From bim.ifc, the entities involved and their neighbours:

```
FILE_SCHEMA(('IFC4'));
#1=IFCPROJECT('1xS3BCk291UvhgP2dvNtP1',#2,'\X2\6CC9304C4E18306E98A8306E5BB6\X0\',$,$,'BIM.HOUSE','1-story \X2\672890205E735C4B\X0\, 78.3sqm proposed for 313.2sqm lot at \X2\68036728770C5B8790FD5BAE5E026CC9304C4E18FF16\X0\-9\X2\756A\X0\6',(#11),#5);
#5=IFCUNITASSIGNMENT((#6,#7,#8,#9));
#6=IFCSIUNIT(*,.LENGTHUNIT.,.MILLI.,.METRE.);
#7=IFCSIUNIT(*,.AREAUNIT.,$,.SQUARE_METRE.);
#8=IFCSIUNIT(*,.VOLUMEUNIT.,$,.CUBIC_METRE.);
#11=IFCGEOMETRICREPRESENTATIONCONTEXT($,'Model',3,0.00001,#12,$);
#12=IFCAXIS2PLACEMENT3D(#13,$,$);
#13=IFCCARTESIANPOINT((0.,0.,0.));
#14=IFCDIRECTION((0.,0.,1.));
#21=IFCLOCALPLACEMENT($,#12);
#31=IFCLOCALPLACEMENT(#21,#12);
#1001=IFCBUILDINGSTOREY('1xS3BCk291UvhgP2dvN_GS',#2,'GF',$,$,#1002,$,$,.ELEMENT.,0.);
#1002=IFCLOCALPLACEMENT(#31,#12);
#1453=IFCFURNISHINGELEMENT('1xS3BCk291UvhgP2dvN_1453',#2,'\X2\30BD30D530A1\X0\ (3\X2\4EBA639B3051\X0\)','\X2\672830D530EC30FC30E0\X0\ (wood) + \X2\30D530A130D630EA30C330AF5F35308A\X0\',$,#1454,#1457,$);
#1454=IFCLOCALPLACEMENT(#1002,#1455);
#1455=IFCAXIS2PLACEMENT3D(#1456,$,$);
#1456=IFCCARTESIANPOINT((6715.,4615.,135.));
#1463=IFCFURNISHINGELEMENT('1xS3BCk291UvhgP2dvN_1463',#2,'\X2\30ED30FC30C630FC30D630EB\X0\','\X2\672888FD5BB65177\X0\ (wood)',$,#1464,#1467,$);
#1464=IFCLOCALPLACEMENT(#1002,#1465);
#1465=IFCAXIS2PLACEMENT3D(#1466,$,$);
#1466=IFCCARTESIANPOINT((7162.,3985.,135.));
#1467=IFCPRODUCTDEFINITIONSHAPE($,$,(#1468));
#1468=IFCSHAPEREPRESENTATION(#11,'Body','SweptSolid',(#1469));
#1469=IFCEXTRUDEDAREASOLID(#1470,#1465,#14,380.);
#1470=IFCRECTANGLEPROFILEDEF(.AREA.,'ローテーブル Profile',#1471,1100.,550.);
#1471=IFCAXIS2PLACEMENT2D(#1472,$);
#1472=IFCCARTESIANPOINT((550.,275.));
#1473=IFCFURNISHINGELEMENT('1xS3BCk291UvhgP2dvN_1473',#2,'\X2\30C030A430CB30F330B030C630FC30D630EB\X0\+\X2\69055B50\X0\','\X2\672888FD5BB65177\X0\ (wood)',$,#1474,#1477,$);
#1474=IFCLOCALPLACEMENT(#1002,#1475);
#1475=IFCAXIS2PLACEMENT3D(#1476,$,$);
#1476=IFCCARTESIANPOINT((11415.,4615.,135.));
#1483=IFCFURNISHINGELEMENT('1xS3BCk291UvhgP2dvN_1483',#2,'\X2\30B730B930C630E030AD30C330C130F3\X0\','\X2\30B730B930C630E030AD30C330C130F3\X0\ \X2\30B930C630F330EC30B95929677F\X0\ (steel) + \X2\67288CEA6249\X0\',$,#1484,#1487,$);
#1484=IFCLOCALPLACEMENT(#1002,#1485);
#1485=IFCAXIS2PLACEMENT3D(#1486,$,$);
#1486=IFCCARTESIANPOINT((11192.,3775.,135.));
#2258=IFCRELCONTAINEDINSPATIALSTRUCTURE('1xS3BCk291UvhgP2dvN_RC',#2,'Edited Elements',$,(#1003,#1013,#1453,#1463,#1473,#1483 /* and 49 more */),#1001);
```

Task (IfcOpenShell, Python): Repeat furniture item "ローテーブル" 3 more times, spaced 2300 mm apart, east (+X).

```python
import numpy as np
import ifcopenshell
import ifcopenshell.api.geometry
import ifcopenshell.api.root
import ifcopenshell.util.element
import ifcopenshell.util.placement
import ifcopenshell.util.unit

model = ifcopenshell.open("bim.ifc")
unit_scale = ifcopenshell.util.unit.calculate_unit_scale(model)


def reuse_history(source, copy):
    """copy_class also copies each property set's owner history, people and application; keep the originals."""
    for rel in copy.IsDefinedBy:
        if rel.is_a("IfcRelDefinesByProperties") and (history := rel.RelatingPropertyDefinition.OwnerHistory):
            rel.RelatingPropertyDefinition.OwnerHistory = source.OwnerHistory
            ifcopenshell.util.element.remove_deep2(model, history)


source = model.by_guid("1xS3BCk291UvhgP2dvN_1463")
base = ifcopenshell.util.placement.get_local_placement(source.ObjectPlacement)
step = np.array([1.0, 0.0, 0.0]) * 2.3 / unit_scale

for i in range(1, 4):
    copy = ifcopenshell.api.root.copy_class(model, product=source)
    copy.Representation = ifcopenshell.util.element.copy_deep(
        model, source.Representation, exclude=["IfcGeometricRepresentationContext", "IfcRepresentationMap"]
    )
    reuse_history(source, copy)
    matrix = base.copy()
    matrix[:3, 3] += i * step
    print("added at", matrix[:3, 3].round(3) + 0.0)
    ifcopenshell.api.geometry.edit_object_placement(model, product=copy, matrix=matrix, is_si=False)

model.write("bim_v2.ifc")
```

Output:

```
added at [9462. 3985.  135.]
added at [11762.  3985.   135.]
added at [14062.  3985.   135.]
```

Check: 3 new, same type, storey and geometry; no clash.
